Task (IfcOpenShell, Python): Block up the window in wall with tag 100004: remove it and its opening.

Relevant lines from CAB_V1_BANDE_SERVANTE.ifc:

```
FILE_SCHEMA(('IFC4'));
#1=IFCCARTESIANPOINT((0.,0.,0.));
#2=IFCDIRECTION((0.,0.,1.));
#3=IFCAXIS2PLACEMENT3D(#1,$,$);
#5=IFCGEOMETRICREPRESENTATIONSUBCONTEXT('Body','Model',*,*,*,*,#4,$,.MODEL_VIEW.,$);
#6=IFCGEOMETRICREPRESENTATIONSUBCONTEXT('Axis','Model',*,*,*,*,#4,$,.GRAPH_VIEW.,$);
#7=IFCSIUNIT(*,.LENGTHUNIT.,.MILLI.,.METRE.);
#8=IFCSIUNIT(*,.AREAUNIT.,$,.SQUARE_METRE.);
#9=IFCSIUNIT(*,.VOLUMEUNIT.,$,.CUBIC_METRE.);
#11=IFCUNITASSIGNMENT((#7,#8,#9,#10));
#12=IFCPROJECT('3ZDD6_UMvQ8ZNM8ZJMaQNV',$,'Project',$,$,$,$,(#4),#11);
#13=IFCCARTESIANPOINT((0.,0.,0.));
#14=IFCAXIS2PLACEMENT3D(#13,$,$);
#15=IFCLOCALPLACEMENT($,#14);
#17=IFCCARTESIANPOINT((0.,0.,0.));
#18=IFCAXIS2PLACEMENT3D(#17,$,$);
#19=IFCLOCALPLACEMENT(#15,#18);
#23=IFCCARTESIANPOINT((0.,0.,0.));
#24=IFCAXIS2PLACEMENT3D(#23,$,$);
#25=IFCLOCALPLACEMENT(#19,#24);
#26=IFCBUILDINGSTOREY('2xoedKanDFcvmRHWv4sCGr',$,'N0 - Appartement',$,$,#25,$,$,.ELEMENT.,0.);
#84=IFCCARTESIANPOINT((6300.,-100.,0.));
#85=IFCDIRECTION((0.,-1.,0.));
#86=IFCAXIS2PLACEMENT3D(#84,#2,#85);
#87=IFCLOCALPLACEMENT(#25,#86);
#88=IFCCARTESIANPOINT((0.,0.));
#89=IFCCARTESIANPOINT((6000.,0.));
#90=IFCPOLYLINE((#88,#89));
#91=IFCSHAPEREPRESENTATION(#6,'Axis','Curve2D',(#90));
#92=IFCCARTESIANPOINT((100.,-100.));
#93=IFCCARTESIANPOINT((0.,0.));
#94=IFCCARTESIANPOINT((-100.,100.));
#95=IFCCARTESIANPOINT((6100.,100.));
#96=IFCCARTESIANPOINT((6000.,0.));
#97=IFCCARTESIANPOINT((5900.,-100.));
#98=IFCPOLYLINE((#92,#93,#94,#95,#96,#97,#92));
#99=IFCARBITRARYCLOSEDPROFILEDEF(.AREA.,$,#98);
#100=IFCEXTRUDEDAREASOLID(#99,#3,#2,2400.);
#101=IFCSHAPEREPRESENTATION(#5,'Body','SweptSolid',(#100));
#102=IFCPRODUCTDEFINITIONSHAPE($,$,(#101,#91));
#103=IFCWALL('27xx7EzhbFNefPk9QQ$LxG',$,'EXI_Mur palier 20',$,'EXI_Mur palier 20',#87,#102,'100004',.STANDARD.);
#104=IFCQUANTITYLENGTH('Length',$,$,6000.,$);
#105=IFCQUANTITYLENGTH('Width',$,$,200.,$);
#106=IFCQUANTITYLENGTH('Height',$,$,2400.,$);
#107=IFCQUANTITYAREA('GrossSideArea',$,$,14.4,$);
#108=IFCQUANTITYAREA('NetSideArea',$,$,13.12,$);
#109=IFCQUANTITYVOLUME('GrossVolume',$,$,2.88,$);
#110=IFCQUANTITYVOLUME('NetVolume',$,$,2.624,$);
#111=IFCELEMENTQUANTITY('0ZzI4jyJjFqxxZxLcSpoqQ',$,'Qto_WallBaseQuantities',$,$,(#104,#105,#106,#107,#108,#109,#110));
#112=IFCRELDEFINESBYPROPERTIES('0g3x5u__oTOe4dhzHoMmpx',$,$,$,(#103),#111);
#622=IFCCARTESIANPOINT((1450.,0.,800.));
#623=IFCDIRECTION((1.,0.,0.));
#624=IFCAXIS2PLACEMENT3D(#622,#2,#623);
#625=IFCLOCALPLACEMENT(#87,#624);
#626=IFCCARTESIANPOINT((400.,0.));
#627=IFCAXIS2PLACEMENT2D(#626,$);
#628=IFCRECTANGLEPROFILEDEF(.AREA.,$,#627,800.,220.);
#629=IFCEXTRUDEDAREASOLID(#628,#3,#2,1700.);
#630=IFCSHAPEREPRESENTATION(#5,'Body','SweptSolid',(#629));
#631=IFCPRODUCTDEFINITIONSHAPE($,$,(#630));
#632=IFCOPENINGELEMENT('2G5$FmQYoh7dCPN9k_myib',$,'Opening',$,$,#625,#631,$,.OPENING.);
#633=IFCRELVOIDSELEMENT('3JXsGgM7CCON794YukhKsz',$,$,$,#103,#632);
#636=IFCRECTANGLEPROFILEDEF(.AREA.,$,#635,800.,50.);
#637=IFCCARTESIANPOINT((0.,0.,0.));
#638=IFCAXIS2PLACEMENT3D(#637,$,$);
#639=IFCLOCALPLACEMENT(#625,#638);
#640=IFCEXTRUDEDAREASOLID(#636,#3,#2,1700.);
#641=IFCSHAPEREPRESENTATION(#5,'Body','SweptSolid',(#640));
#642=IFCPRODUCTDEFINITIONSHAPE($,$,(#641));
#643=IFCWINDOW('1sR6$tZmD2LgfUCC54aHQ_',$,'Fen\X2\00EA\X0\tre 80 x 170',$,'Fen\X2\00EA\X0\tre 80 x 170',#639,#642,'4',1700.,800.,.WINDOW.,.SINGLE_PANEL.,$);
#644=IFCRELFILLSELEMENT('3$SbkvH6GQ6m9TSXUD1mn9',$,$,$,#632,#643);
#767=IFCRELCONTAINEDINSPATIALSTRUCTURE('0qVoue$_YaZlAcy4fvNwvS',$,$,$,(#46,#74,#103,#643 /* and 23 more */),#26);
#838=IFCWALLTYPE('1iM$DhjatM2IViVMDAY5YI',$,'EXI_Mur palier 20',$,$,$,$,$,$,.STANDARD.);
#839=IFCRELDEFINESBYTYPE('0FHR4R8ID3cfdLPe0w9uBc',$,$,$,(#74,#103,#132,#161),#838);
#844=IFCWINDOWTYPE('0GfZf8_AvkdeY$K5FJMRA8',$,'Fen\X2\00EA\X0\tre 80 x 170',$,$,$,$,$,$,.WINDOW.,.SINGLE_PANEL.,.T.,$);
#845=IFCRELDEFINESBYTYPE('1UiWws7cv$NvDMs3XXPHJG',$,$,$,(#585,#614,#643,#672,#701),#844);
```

```python
import ifcopenshell
import ifcopenshell.api.feature
import ifcopenshell.api.pset
import ifcopenshell.api.root
import ifcopenshell.geom
import ifcopenshell.util.element
import ifcopenshell.util.shape
import ifcopenshell.util.unit

model = ifcopenshell.open("CAB_V1_BANDE_SERVANTE.ifc")
area_scale = ifcopenshell.util.unit.calculate_unit_scale(model, "AREAUNIT")
volume_scale = ifcopenshell.util.unit.calculate_unit_scale(model, "VOLUMEUNIT")
settings = ifcopenshell.geom.settings()


def volume(element):
    """Net volume in cubic metres, openings subtracted."""
    shape = ifcopenshell.geom.create_shape(settings, element)
    return ifcopenshell.util.shape.get_volume(shape.geometry)


window = model.by_guid("1sR6$tZmD2LgfUCC54aHQ_")
opening = window.FillsVoids[0].RelatingOpeningElement
wall = opening.VoidsElements[0].RelatingBuildingElement
before = volume(wall)

ifcopenshell.api.root.remove_product(model, product=window)
ifcopenshell.api.feature.remove_feature(model, feature=opening)

after = volume(wall)
thickness = 0.2  # wall thickness in metres

# Update the wall's stored quantities.
qto = model.by_id(ifcopenshell.util.element.get_pset(wall, "Qto_WallBaseQuantities", should_inherit=False)["id"])
ifcopenshell.api.pset.edit_qto(model, qto=qto, properties={
    "NetSideArea": after / thickness / area_scale,
    "NetVolume": after / volume_scale,
})

print(f"wall volume {before:.3f} -> {after:.3f} m3")

model.write("CAB_V1_BANDE_SERVANTE-out.ifc")
```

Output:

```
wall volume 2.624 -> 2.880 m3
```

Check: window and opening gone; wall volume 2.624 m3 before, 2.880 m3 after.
